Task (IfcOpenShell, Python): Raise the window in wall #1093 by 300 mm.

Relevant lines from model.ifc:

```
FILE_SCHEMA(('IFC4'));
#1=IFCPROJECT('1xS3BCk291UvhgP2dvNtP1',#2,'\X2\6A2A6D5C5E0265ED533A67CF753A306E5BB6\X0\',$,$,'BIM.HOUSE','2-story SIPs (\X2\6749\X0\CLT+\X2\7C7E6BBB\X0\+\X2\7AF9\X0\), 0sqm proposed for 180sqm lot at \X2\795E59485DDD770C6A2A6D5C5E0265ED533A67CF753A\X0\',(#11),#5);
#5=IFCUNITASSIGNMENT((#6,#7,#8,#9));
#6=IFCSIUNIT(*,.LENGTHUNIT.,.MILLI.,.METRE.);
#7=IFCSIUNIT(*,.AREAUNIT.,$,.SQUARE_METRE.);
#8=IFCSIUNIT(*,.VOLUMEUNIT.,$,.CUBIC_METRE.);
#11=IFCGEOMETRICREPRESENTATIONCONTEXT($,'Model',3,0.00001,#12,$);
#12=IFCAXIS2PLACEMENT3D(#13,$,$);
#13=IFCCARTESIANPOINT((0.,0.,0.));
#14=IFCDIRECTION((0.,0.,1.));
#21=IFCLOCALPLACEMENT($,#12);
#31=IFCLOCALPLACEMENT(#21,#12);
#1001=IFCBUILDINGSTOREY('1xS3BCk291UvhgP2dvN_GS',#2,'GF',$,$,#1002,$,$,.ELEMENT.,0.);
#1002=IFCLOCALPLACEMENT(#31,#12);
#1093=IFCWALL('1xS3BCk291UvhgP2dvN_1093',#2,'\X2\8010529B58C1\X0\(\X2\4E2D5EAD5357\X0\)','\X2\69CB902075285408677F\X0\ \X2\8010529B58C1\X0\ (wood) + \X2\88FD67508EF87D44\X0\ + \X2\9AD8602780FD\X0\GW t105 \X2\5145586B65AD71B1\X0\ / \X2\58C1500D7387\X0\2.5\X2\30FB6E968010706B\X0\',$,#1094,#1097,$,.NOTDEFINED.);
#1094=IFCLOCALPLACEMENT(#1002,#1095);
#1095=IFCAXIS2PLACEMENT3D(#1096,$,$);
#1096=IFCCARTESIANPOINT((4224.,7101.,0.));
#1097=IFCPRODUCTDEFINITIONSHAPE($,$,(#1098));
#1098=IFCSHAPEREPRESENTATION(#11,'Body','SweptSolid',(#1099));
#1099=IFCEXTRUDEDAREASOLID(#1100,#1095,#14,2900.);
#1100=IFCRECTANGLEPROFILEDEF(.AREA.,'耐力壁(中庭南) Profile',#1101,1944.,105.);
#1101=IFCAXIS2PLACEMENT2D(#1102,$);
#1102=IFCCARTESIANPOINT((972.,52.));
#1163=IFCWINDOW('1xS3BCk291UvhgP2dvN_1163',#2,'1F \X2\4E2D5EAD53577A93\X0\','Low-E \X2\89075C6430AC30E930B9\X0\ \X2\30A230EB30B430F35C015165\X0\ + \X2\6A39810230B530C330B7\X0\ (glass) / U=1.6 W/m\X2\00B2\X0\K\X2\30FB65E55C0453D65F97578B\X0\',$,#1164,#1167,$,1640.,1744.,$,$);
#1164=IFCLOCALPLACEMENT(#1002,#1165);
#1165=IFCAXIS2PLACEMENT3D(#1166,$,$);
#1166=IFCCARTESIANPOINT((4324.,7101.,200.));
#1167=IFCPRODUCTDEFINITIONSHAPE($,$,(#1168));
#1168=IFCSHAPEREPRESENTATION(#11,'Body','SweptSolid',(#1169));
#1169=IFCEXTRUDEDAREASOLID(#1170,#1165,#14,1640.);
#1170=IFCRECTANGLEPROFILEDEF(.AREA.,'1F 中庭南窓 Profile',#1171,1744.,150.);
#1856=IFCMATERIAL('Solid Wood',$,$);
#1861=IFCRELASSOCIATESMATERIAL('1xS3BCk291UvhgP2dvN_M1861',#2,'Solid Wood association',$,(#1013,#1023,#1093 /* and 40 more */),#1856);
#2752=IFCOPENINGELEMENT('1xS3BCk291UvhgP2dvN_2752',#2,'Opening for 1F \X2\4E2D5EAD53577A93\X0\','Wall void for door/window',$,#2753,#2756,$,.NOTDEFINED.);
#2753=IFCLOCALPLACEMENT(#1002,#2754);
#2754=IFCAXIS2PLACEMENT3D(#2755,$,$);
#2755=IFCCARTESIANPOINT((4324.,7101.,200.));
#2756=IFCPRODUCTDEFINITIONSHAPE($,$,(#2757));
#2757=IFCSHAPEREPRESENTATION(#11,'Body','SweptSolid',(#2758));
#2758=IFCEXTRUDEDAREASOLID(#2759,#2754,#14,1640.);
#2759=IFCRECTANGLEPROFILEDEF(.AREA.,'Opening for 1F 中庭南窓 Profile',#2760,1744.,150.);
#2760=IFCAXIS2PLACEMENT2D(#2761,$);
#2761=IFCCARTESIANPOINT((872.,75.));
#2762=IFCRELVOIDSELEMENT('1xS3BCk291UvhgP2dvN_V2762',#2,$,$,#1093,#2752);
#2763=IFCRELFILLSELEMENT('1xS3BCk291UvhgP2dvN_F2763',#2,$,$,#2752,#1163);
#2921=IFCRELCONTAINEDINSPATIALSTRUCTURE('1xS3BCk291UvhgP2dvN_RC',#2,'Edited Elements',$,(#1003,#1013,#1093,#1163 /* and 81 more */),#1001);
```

```python
import numpy as np
import ifcopenshell
import ifcopenshell.api.geometry
import ifcopenshell.util.placement
import ifcopenshell.util.unit

model = ifcopenshell.open("model.ifc")
unit_scale = ifcopenshell.util.unit.calculate_unit_scale(model)

window = model.by_id(1163)
opening = window.FillsVoids[0].RelatingOpeningElement
dz = 0.3 / unit_scale

shift = np.array([0.0, 0.0, dz])
# The window is not placed relative to its opening, so move both.
for product in (opening, window):
    matrix = ifcopenshell.util.placement.get_local_placement(product.ObjectPlacement)
    matrix[:3, 3] += shift
    ifcopenshell.api.geometry.edit_object_placement(model, product=product, matrix=matrix, is_si=False)

print(f"moved by {dz * unit_scale:+.3f} m")

model.write("model_edited.ifc")
```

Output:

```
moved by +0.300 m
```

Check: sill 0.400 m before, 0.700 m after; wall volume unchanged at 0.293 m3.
